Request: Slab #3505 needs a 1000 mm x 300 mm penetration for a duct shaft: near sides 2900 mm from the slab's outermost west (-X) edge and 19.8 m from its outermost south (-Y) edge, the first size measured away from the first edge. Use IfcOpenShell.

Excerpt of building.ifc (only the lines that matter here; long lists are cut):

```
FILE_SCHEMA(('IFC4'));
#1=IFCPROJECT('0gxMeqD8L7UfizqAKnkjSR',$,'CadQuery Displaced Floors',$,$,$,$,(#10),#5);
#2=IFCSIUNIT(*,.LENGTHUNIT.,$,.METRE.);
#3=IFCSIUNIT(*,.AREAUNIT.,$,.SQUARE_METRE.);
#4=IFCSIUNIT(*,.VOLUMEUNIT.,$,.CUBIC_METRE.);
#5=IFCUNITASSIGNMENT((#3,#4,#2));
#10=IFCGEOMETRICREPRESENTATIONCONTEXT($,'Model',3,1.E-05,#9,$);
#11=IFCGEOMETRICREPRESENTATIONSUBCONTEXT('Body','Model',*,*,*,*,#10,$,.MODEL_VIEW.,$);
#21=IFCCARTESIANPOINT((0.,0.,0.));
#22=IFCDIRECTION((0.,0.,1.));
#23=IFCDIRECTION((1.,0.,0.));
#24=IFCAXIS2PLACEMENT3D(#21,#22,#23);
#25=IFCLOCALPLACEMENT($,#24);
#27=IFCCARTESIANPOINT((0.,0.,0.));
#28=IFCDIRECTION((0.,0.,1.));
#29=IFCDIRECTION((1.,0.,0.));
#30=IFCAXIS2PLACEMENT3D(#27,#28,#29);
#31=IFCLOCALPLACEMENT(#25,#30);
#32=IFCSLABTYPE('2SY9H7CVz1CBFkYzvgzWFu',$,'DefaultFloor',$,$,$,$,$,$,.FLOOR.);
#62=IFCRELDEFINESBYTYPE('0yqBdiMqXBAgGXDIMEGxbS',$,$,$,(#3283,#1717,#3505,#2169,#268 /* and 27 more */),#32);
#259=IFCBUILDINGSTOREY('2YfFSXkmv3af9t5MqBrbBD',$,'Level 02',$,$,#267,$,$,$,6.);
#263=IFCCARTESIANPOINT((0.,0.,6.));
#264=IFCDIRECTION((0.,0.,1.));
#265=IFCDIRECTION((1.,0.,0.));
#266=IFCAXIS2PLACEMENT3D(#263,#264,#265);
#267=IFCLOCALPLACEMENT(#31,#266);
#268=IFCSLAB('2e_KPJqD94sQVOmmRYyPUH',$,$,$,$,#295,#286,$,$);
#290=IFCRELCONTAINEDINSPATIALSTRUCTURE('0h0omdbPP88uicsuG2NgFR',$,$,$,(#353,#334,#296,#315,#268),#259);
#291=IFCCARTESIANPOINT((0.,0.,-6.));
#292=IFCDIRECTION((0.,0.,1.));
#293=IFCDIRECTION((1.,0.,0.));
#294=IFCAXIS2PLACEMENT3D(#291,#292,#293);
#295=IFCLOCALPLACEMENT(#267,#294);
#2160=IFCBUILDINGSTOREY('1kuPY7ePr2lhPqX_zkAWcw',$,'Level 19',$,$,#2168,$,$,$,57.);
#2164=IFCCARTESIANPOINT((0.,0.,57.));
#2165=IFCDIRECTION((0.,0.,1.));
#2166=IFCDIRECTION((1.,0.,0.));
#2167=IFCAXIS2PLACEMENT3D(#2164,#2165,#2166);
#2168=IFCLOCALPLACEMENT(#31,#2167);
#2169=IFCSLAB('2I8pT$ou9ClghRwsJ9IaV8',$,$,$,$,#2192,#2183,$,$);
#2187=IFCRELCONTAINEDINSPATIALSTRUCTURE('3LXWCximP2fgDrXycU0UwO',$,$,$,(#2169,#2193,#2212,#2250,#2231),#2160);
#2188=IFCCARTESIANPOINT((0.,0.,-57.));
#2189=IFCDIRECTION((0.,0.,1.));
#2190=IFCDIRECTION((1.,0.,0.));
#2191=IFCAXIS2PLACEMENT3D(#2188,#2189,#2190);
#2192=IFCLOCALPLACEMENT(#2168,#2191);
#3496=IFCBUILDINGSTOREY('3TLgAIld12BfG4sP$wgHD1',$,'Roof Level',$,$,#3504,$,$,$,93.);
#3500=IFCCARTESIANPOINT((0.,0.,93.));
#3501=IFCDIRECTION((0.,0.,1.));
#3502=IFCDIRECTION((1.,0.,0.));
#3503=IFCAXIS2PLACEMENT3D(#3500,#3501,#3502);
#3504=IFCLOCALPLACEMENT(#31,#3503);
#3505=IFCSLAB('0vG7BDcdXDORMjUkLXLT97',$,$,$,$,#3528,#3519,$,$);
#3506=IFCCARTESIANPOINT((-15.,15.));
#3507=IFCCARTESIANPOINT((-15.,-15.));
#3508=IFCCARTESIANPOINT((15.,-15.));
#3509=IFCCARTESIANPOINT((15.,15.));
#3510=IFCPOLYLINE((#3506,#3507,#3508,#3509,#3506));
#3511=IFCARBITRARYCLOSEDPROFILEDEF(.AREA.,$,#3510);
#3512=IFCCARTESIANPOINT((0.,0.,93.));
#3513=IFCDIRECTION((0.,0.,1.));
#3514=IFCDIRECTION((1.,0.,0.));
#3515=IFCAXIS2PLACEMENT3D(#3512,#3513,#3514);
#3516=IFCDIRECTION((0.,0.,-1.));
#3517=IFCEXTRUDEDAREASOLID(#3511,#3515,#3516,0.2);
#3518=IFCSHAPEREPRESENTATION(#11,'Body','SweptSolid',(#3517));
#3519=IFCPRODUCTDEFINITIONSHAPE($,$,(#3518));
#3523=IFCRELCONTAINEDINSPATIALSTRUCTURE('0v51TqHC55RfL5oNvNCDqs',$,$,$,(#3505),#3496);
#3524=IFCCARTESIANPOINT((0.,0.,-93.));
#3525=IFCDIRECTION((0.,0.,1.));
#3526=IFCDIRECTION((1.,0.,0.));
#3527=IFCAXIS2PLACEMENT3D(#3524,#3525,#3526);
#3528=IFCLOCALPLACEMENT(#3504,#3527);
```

```python
import numpy as np
import ifcopenshell
import ifcopenshell.api.feature
import ifcopenshell.api.geometry
import ifcopenshell.api.root
import ifcopenshell.geom
import ifcopenshell.util.placement
import ifcopenshell.util.representation
import ifcopenshell.util.shape
import ifcopenshell.util.unit

model = ifcopenshell.open("building.ifc")
unit_scale = ifcopenshell.util.unit.calculate_unit_scale(model)
settings = ifcopenshell.geom.settings()


def volume(element):
    """Net volume in cubic metres, openings subtracted."""
    shape = ifcopenshell.geom.create_shape(settings, element)
    return ifcopenshell.util.shape.get_volume(shape.geometry)


slab = model.by_guid("0vG7BDcdXDORMjUkLXLT97")
before = volume(slab)

# Extent in the slab's own axes, in metres. The edges named are its -X and -Y sides.
slab_shape = ifcopenshell.geom.create_shape(settings, slab)
vertices = ifcopenshell.util.shape.get_vertices(slab_shape.geometry)
x_min, y_min, bottom = vertices.min(axis=0)
top = vertices[:, 2].max()

opening = ifcopenshell.api.root.create_entity(model, ifc_class="IfcOpeningElement", name="Duct shaft opening", predefined_type="OPENING")
context = ifcopenshell.util.representation.get_context(model, "Model", "Body", "MODEL_VIEW")
width, depth = 1, 0.3
outline = [(0.0, 0.0), (width, 0.0), (width, depth), (0.0, depth), (0.0, 0.0)]
# Overshoot both faces by 50 mm so the cut is clean.
shape = ifcopenshell.api.geometry.add_slab_representation(
    model, context=context, depth=top - bottom + 0.1, polyline=outline
)
ifcopenshell.api.geometry.assign_representation(model, product=opening, representation=shape)

matrix = ifcopenshell.util.placement.get_local_placement(slab.ObjectPlacement)
matrix[:, 3] = matrix @ np.append(np.array([x_min + 2.9, y_min + 19.8, bottom - 0.05]) / unit_scale, 1.0)
ifcopenshell.api.geometry.edit_object_placement(model, product=opening, matrix=matrix, is_si=False)
ifcopenshell.api.feature.add_feature(model, feature=opening, element=slab)

after = volume(slab)

print(f"slab volume {before:.3f} -> {after:.3f} m3")

model.write("building_edited.ifc")
```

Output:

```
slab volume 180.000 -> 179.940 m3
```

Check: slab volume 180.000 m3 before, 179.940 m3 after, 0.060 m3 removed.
